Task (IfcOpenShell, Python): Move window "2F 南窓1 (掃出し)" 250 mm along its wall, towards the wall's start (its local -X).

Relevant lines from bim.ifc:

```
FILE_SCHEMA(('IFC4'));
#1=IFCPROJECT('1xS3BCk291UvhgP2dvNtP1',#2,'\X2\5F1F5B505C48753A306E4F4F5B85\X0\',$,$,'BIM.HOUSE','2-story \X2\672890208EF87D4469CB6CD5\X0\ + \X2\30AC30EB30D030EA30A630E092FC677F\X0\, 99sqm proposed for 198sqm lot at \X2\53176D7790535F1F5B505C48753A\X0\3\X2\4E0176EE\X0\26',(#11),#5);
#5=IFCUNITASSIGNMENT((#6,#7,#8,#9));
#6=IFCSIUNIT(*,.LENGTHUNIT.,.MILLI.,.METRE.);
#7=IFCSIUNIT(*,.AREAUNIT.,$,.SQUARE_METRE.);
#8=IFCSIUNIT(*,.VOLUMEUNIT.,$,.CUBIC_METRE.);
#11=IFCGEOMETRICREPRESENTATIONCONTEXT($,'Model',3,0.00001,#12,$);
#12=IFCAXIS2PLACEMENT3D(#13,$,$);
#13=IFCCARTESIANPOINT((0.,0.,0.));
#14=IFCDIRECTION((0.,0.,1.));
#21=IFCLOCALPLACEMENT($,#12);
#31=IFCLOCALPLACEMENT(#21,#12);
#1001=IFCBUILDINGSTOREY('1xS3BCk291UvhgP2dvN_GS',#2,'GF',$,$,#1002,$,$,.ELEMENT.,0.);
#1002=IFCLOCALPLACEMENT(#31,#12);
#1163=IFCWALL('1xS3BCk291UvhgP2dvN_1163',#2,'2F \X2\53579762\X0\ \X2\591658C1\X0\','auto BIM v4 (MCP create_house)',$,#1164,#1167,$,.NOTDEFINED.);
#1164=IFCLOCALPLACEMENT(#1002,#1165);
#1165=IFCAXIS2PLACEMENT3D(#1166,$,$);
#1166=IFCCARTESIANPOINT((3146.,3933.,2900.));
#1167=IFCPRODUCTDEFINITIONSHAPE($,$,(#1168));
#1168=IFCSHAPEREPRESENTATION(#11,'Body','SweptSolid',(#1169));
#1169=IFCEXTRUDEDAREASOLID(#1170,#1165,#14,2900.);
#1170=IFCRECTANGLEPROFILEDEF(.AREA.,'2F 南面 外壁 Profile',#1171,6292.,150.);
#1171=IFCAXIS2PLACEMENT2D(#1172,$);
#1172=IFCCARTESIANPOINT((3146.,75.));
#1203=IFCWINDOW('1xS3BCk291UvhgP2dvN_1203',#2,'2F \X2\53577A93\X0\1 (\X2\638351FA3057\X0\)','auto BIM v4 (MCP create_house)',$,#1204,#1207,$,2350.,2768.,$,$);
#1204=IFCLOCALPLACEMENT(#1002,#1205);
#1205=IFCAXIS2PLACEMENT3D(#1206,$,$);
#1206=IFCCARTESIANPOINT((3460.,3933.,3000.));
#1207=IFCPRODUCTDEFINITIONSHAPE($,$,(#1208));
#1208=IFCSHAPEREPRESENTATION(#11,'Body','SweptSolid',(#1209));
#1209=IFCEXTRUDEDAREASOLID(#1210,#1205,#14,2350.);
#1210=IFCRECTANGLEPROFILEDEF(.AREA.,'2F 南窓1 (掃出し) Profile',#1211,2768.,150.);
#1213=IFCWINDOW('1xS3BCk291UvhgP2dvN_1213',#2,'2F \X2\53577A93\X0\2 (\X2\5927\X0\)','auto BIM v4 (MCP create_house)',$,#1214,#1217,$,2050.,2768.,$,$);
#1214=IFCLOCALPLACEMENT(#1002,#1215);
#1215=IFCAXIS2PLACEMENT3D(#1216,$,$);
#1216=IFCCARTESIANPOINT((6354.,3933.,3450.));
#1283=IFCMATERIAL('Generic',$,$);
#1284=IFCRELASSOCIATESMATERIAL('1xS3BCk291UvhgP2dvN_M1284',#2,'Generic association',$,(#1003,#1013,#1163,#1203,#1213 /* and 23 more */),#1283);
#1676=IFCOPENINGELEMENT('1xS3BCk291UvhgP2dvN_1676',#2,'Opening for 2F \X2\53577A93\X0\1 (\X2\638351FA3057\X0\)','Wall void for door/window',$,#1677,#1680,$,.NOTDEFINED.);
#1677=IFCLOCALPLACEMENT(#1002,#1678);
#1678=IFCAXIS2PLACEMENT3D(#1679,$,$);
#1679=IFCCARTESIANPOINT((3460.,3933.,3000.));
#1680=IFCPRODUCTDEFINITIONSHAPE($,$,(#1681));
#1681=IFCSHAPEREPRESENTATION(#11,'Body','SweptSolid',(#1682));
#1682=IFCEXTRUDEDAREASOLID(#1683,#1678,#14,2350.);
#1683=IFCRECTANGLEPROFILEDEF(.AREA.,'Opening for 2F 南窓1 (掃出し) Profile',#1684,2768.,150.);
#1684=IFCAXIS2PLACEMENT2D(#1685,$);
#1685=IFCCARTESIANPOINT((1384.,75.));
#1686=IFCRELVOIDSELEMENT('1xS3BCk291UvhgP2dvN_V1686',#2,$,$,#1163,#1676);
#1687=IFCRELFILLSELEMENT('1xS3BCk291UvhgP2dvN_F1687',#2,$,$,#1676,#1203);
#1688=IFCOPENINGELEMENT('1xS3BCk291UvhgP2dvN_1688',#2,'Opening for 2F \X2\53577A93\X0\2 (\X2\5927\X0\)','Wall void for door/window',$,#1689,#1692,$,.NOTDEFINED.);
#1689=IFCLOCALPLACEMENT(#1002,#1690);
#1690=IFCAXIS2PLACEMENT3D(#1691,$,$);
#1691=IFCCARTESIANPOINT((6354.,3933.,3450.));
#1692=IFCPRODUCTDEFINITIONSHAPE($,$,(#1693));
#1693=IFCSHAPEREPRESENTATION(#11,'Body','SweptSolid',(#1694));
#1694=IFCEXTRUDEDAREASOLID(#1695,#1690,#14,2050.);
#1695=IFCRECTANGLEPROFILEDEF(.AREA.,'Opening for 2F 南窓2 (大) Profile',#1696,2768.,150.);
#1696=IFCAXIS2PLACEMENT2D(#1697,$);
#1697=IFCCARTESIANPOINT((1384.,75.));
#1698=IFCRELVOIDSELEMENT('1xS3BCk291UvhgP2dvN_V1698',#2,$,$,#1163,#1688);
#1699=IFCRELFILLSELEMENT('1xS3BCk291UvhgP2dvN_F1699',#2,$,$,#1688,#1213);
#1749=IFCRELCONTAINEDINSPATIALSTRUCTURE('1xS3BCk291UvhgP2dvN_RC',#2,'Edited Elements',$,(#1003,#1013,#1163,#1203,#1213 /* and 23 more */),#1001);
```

```python
import ifcopenshell
import ifcopenshell.api.geometry
import ifcopenshell.util.placement

model = ifcopenshell.open("bim.ifc")

window = model.by_guid("1xS3BCk291UvhgP2dvN_1203")
opening = window.FillsVoids[0].RelatingOpeningElement
wall = opening.VoidsElements[0].RelatingBuildingElement

wall_matrix = ifcopenshell.util.placement.get_local_placement(wall.ObjectPlacement)
shift = wall_matrix[:3, 0] * -250.0
before = ifcopenshell.util.placement.get_local_placement(window.ObjectPlacement)[:3, 3].copy()

# The window is not placed relative to its opening, so move both.
for product in (opening, window):
    matrix = ifcopenshell.util.placement.get_local_placement(product.ObjectPlacement)
    matrix[:3, 3] += shift
    ifcopenshell.api.geometry.edit_object_placement(model, product=product, matrix=matrix, is_si=False)

after = ifcopenshell.util.placement.get_local_placement(window.ObjectPlacement)[:3, 3]
print("window moved by", (after - before).round(3) + 0.0)

model.write("bim_edited.ifc")
```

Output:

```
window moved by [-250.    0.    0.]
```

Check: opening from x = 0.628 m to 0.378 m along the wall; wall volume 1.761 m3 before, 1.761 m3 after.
